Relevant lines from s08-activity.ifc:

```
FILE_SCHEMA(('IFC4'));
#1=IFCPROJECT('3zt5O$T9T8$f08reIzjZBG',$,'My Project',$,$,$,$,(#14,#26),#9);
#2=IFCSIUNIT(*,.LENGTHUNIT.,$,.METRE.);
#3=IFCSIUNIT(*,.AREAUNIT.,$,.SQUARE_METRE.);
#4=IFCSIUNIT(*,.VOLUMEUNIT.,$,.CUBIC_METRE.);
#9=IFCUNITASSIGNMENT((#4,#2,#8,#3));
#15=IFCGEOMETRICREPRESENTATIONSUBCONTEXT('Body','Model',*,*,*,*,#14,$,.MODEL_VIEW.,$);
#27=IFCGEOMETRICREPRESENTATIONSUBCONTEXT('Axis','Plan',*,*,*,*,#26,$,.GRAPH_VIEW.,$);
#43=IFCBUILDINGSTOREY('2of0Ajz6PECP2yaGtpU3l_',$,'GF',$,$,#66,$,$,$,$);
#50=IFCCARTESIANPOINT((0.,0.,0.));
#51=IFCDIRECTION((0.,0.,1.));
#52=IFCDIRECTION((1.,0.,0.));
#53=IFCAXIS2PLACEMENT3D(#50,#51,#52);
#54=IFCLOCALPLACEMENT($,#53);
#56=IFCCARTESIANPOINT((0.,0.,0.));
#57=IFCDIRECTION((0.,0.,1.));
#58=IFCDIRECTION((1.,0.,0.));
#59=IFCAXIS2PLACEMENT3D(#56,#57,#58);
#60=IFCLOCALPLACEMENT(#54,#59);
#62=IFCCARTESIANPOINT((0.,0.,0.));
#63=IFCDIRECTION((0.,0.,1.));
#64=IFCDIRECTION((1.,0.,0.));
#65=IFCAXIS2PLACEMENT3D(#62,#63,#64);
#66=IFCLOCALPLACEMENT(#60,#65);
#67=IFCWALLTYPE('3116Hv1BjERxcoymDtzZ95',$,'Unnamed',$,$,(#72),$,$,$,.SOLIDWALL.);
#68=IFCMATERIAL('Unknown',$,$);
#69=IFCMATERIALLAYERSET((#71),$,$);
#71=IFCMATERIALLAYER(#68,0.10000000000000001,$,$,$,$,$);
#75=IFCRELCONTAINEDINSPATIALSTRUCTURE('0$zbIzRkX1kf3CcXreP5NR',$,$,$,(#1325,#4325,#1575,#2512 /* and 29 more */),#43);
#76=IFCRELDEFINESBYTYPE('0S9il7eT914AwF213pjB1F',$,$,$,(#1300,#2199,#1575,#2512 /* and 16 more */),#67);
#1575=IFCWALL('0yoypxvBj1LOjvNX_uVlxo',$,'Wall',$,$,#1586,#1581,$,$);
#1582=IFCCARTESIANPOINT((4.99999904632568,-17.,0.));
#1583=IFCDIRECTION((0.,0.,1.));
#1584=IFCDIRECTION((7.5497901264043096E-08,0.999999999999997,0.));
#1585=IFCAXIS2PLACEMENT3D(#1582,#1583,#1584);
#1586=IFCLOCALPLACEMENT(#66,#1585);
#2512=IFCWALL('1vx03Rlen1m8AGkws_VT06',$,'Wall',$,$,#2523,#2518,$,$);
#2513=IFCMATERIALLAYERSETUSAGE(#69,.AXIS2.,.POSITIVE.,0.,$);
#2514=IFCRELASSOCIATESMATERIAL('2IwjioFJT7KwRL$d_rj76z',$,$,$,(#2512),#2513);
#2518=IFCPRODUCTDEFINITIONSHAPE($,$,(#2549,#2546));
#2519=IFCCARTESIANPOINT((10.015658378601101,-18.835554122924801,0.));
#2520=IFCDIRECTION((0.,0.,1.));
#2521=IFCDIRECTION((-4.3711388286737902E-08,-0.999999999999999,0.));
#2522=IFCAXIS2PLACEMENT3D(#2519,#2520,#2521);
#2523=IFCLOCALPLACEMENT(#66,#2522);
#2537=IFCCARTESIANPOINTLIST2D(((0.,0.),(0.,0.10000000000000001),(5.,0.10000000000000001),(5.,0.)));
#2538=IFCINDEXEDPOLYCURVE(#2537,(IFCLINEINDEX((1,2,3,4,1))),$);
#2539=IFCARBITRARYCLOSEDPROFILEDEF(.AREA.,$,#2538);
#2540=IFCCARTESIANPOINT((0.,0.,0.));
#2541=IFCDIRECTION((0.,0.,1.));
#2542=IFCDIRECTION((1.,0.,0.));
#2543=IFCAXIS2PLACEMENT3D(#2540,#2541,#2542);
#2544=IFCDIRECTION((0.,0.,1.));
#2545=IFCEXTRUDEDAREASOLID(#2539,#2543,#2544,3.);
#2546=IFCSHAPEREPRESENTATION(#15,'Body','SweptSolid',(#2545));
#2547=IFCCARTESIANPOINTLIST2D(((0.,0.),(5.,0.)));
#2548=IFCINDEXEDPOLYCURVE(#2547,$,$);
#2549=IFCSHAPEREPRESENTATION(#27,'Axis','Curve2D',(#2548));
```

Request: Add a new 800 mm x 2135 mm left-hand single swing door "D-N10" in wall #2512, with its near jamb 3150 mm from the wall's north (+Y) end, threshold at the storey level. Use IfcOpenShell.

```python
import numpy as np
import ifcopenshell
import ifcopenshell.api.feature
import ifcopenshell.api.geometry
import ifcopenshell.api.root
import ifcopenshell.api.spatial
import ifcopenshell.geom
import ifcopenshell.util.element
import ifcopenshell.util.placement
import ifcopenshell.util.representation
import ifcopenshell.util.shape
import ifcopenshell.util.unit

model = ifcopenshell.open("s08-activity.ifc")
unit_scale = ifcopenshell.util.unit.calculate_unit_scale(model)
settings = ifcopenshell.geom.settings()


def volume(element):
    """Net volume in cubic metres, openings subtracted."""
    shape = ifcopenshell.geom.create_shape(settings, element)
    return ifcopenshell.util.shape.get_volume(shape.geometry)


wall = model.by_guid("1vx03Rlen1m8AGkws_VT06")
storey = ifcopenshell.util.element.get_container(wall, ifc_class="IfcBuildingStorey")
context = ifcopenshell.util.representation.get_context(model, "Model", "Body", "MODEL_VIEW")
before = volume(wall)

width, height, from_end, sill = 0.8, 2.135, 3.15, 0.0  # metres

# The wall runs along its own X axis, and the end named is its -X end.
wall_shape = ifcopenshell.geom.create_shape(settings, wall)
x, y, z = ifcopenshell.util.shape.get_vertices(wall_shape.geometry).T
start = x.min() + from_end
face, thickness = float(y.min()), float(y.max() - y.min())
wall_matrix = ifcopenshell.util.placement.get_local_placement(wall.ObjectPlacement)
level = ifcopenshell.util.placement.get_local_placement(storey.ObjectPlacement)[2, 3]


def in_wall(x, y):
    """Placement at x, y metres in the wall's axes, at sill height."""
    matrix = wall_matrix.copy()
    matrix[:, 3] = wall_matrix @ np.array([x / unit_scale, y / unit_scale, 0.0, 1.0])
    matrix[2, 3] = level + sill / unit_scale
    return matrix


# Opening: a box that overshoots both wall faces by 50 mm.
opening = ifcopenshell.api.root.create_entity(model, ifc_class="IfcOpeningElement", predefined_type="OPENING")
box = ifcopenshell.api.geometry.add_wall_representation(
    model, context=context, length=width, height=height, thickness=thickness + 0.1
)
ifcopenshell.api.geometry.assign_representation(model, product=opening, representation=box)
ifcopenshell.api.geometry.edit_object_placement(model, product=opening, matrix=in_wall(start, face - 0.05), is_si=False)
ifcopenshell.api.feature.add_feature(model, feature=opening, element=wall)

door = ifcopenshell.api.root.create_entity(model, ifc_class="IfcDoor", name="D-N10", predefined_type="DOOR")
door.OverallWidth, door.OverallHeight = width / unit_scale, height / unit_scale
door.OperationType = "SINGLE_SWING_LEFT"
body = ifcopenshell.api.geometry.add_door_representation(
    model,
    context=context,
    overall_width=door.OverallWidth,
    overall_height=door.OverallHeight,
    operation_type="SINGLE_SWING_LEFT",
    lining_properties={"LiningDepth": thickness / unit_scale, "ThresholdDepth": thickness / unit_scale},
)
ifcopenshell.api.geometry.assign_representation(model, product=door, representation=body)
ifcopenshell.api.spatial.assign_container(model, products=[door], relating_structure=storey)
ifcopenshell.api.feature.add_filling(model, opening=opening, element=door)

# The lining spans the wall, so the door starts at the wall face.
ifcopenshell.api.geometry.edit_object_placement(model, product=door, matrix=in_wall(start, face), is_si=False)

after = volume(wall)

print(f"wall volume {before:.3f} -> {after:.3f} m3")

model.write("s08-activity_rev.ifc")
```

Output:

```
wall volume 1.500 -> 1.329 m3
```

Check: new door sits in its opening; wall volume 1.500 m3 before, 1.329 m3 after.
